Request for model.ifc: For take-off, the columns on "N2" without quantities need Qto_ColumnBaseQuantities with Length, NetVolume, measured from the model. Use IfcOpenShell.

First a look at what the model holds.

```python
import ifcopenshell
import ifcopenshell.util.element
import ifcopenshell.util.unit

model = ifcopenshell.open("model.ifc")
print(model.schema)
for unit_type in ("LENGTHUNIT", "AREAUNIT", "VOLUMEUNIT"):
    print(unit_type, ifcopenshell.util.unit.calculate_unit_scale(model, unit_type))
storey = next(s for s in model.by_type("IfcBuildingStorey") if s.Name == "N2")
columns = [e for e in ifcopenshell.util.element.get_decomposition(storey) if e.is_a("IfcColumn")]
for e in sorted(columns, key=lambda e: e.id()):
    print(e.id(), e.is_a(), e.Name, list(ifcopenshell.util.element.get_psets(e, qtos_only=True)), sep=" | ")
```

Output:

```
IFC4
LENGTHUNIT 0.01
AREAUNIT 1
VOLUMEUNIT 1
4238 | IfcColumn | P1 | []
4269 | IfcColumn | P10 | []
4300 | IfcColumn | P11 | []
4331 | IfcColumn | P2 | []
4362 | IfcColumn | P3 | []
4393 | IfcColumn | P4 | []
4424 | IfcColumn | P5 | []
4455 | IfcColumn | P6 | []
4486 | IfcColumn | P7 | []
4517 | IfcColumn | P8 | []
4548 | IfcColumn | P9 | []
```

```python
import ifcopenshell
import ifcopenshell.api.pset
import ifcopenshell.geom
import ifcopenshell.util.element
import ifcopenshell.util.shape
import ifcopenshell.util.unit

model = ifcopenshell.open("model.ifc")
unit_scale = ifcopenshell.util.unit.calculate_unit_scale(model)
volume_scale = ifcopenshell.util.unit.calculate_unit_scale(model, "VOLUMEUNIT")
settings = ifcopenshell.geom.settings()

storey = next(s for s in model.by_type("IfcBuildingStorey") if s.Name == "N2")
columns = [e for e in ifcopenshell.util.element.get_decomposition(storey) if e.is_a("IfcColumn")]

for e in sorted(columns, key=lambda e: e.id()):
    if ifcopenshell.util.element.get_psets(e, qtos_only=True, should_inherit=False):
        continue
    # Geometry comes back in metres, in the element's own axes.
    shape = ifcopenshell.geom.create_shape(settings, e)
    values = {
        "Length": ifcopenshell.util.shape.get_z(shape.geometry) / unit_scale,
        "NetVolume": ifcopenshell.util.shape.get_volume(shape.geometry) / volume_scale,
    }
    qto = ifcopenshell.api.pset.add_qto(model, product=e, name="Qto_ColumnBaseQuantities")
    ifcopenshell.api.pset.edit_qto(model, qto=qto, properties=values)
    print(e.id(), {k: round(v, 3) for k, v in values.items()})

model.write("model_edited.ifc")
```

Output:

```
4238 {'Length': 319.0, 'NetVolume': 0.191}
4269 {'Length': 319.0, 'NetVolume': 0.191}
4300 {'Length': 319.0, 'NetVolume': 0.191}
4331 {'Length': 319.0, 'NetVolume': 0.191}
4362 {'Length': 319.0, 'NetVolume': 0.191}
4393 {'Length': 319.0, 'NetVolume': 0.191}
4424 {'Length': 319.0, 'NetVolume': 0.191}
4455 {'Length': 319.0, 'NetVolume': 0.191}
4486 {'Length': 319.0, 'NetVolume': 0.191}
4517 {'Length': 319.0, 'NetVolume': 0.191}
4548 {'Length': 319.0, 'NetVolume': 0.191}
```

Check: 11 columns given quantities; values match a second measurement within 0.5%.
